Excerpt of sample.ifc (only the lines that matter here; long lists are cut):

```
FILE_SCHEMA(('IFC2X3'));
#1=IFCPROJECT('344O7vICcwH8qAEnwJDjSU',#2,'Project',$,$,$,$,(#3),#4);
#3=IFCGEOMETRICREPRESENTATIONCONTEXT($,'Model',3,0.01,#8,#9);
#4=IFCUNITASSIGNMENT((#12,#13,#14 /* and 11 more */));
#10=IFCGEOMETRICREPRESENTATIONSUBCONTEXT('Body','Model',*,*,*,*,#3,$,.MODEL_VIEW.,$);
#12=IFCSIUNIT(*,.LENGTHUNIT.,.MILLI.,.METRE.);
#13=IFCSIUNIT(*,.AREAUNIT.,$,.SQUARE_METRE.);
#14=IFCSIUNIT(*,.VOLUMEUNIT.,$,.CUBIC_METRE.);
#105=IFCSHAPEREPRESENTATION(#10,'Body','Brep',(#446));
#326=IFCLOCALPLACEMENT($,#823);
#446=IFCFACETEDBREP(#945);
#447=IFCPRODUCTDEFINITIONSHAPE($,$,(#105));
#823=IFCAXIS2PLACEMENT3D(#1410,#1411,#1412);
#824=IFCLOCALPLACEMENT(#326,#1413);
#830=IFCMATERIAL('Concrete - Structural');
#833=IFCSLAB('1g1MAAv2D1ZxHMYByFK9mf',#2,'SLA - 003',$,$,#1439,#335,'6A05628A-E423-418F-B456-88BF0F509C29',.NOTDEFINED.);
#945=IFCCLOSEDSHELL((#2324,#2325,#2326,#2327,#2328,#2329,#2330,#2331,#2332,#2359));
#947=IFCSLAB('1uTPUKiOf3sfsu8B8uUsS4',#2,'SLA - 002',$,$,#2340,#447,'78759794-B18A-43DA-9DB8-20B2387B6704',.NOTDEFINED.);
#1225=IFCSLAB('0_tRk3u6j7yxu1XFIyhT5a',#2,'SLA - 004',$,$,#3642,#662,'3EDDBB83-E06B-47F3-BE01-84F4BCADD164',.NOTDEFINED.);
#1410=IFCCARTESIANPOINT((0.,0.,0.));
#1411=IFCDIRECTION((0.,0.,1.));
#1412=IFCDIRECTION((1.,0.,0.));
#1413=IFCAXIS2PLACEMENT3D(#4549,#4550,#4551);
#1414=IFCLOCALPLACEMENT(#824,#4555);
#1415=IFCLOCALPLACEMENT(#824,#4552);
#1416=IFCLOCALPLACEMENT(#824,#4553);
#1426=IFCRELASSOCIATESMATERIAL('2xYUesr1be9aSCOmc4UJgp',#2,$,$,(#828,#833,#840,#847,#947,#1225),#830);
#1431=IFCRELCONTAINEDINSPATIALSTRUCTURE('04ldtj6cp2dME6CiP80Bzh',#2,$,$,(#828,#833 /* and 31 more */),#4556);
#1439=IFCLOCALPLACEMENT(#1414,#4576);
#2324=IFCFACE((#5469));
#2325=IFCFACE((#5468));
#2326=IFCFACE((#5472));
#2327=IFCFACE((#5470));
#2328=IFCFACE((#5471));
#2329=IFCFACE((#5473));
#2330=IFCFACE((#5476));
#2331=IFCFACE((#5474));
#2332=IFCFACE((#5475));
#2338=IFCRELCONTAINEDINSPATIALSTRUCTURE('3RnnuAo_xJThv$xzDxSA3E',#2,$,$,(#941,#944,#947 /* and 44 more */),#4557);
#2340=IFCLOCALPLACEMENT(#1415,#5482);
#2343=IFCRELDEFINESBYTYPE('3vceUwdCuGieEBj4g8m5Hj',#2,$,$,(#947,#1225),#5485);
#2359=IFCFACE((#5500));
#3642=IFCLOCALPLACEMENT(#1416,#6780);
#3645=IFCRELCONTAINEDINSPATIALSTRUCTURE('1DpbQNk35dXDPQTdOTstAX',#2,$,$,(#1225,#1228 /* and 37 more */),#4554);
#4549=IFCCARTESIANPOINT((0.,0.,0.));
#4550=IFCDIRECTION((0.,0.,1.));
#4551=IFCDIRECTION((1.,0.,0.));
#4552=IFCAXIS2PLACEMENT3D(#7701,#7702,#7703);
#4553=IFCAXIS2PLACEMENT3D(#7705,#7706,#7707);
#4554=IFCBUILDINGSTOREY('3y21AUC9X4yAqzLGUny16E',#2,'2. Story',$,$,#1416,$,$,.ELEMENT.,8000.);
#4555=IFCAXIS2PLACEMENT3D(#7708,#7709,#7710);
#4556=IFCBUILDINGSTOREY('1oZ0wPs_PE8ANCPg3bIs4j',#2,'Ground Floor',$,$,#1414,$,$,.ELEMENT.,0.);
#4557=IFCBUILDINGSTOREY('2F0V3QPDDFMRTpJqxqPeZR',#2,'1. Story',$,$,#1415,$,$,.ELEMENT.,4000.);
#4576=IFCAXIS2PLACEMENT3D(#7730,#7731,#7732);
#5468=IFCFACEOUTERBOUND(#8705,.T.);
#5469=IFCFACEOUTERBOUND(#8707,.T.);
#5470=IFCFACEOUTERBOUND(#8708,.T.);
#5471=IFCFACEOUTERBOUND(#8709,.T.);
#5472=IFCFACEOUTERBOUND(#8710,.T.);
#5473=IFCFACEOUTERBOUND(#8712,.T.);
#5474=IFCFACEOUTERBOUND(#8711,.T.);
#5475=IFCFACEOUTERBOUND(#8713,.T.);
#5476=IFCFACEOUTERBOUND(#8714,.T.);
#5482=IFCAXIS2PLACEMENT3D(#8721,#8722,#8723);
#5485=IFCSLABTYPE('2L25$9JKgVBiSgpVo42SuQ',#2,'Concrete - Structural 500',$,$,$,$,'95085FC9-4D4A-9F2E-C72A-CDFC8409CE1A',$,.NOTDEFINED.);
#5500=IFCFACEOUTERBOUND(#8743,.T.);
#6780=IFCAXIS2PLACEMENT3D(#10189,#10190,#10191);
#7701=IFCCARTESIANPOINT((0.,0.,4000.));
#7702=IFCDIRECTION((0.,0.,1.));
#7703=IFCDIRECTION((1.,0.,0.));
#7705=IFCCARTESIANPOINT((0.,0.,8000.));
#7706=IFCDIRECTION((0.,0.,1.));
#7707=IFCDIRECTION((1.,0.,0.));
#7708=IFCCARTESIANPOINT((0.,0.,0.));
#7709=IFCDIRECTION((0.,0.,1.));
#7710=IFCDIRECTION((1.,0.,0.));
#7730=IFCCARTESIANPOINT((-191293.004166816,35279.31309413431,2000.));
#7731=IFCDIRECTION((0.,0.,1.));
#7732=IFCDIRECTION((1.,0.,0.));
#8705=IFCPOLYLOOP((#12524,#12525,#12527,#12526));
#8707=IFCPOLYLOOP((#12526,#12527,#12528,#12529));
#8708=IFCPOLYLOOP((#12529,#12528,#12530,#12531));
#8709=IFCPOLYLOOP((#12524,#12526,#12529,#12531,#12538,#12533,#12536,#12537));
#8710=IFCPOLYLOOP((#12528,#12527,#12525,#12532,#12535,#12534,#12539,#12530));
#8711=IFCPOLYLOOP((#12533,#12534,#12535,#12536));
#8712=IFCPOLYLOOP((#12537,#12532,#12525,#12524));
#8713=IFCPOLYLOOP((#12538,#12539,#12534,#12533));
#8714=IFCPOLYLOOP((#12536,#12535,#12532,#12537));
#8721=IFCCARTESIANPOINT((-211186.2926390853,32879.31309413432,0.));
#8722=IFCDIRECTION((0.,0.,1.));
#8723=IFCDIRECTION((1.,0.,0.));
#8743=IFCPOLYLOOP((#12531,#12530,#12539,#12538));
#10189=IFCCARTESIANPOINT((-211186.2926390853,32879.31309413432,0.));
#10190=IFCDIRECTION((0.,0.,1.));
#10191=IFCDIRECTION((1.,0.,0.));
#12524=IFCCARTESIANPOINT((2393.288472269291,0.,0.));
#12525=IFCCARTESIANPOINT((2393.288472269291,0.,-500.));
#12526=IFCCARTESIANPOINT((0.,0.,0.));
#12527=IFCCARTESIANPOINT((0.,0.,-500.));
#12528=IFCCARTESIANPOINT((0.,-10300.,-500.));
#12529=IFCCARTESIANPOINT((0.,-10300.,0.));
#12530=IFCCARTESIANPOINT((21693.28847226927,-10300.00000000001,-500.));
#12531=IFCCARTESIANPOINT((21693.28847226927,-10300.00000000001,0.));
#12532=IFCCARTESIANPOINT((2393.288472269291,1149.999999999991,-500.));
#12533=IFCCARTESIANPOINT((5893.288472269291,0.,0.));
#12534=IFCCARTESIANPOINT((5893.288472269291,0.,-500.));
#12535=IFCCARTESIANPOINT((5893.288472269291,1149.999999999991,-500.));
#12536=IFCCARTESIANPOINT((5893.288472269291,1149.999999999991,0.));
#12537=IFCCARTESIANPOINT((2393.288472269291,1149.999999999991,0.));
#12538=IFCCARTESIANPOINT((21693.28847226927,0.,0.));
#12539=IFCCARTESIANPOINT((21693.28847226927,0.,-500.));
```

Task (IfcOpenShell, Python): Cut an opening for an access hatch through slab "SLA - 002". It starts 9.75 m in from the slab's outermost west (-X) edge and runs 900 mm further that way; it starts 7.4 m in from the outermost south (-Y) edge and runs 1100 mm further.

```python
import numpy as np
import ifcopenshell
import ifcopenshell.api.feature
import ifcopenshell.api.geometry
import ifcopenshell.api.root
import ifcopenshell.geom
import ifcopenshell.util.placement
import ifcopenshell.util.representation
import ifcopenshell.util.shape
import ifcopenshell.util.unit

model = ifcopenshell.open("sample.ifc")
unit_scale = ifcopenshell.util.unit.calculate_unit_scale(model)
settings = ifcopenshell.geom.settings()


def volume(element):
    """Net volume in cubic metres, openings subtracted."""
    shape = ifcopenshell.geom.create_shape(settings, element)
    return ifcopenshell.util.shape.get_volume(shape.geometry)


slab = model.by_guid("1uTPUKiOf3sfsu8B8uUsS4")
before = volume(slab)

# Extent in the slab's own axes, in metres. The edges named are its -X and -Y sides.
slab_shape = ifcopenshell.geom.create_shape(settings, slab)
vertices = ifcopenshell.util.shape.get_vertices(slab_shape.geometry)
x_min, y_min, bottom = vertices.min(axis=0)
top = vertices[:, 2].max()

opening = ifcopenshell.api.root.create_entity(model, ifc_class="IfcOpeningElement", name="Access hatch opening")
context = ifcopenshell.util.representation.get_context(model, "Model", "Body", "MODEL_VIEW")
width, depth = 0.9, 1.1
outline = [(0.0, 0.0), (width, 0.0), (width, depth), (0.0, depth), (0.0, 0.0)]
# Overshoot both faces by 50 mm so the cut is clean.
shape = ifcopenshell.api.geometry.add_slab_representation(
    model, context=context, depth=top - bottom + 0.1, polyline=outline
)
ifcopenshell.api.geometry.assign_representation(model, product=opening, representation=shape)

matrix = ifcopenshell.util.placement.get_local_placement(slab.ObjectPlacement)
matrix[:, 3] = matrix @ np.append(np.array([x_min + 9.75, y_min + 7.4, bottom - 0.05]) / unit_scale, 1.0)
ifcopenshell.api.geometry.edit_object_placement(model, product=opening, matrix=matrix, is_si=False)
ifcopenshell.api.feature.add_feature(model, feature=opening, element=slab)

after = volume(slab)

print(f"slab volume {before:.3f} -> {after:.3f} m3")

model.write("sample_v2.ifc")
```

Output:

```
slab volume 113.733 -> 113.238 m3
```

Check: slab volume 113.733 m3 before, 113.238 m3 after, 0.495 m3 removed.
